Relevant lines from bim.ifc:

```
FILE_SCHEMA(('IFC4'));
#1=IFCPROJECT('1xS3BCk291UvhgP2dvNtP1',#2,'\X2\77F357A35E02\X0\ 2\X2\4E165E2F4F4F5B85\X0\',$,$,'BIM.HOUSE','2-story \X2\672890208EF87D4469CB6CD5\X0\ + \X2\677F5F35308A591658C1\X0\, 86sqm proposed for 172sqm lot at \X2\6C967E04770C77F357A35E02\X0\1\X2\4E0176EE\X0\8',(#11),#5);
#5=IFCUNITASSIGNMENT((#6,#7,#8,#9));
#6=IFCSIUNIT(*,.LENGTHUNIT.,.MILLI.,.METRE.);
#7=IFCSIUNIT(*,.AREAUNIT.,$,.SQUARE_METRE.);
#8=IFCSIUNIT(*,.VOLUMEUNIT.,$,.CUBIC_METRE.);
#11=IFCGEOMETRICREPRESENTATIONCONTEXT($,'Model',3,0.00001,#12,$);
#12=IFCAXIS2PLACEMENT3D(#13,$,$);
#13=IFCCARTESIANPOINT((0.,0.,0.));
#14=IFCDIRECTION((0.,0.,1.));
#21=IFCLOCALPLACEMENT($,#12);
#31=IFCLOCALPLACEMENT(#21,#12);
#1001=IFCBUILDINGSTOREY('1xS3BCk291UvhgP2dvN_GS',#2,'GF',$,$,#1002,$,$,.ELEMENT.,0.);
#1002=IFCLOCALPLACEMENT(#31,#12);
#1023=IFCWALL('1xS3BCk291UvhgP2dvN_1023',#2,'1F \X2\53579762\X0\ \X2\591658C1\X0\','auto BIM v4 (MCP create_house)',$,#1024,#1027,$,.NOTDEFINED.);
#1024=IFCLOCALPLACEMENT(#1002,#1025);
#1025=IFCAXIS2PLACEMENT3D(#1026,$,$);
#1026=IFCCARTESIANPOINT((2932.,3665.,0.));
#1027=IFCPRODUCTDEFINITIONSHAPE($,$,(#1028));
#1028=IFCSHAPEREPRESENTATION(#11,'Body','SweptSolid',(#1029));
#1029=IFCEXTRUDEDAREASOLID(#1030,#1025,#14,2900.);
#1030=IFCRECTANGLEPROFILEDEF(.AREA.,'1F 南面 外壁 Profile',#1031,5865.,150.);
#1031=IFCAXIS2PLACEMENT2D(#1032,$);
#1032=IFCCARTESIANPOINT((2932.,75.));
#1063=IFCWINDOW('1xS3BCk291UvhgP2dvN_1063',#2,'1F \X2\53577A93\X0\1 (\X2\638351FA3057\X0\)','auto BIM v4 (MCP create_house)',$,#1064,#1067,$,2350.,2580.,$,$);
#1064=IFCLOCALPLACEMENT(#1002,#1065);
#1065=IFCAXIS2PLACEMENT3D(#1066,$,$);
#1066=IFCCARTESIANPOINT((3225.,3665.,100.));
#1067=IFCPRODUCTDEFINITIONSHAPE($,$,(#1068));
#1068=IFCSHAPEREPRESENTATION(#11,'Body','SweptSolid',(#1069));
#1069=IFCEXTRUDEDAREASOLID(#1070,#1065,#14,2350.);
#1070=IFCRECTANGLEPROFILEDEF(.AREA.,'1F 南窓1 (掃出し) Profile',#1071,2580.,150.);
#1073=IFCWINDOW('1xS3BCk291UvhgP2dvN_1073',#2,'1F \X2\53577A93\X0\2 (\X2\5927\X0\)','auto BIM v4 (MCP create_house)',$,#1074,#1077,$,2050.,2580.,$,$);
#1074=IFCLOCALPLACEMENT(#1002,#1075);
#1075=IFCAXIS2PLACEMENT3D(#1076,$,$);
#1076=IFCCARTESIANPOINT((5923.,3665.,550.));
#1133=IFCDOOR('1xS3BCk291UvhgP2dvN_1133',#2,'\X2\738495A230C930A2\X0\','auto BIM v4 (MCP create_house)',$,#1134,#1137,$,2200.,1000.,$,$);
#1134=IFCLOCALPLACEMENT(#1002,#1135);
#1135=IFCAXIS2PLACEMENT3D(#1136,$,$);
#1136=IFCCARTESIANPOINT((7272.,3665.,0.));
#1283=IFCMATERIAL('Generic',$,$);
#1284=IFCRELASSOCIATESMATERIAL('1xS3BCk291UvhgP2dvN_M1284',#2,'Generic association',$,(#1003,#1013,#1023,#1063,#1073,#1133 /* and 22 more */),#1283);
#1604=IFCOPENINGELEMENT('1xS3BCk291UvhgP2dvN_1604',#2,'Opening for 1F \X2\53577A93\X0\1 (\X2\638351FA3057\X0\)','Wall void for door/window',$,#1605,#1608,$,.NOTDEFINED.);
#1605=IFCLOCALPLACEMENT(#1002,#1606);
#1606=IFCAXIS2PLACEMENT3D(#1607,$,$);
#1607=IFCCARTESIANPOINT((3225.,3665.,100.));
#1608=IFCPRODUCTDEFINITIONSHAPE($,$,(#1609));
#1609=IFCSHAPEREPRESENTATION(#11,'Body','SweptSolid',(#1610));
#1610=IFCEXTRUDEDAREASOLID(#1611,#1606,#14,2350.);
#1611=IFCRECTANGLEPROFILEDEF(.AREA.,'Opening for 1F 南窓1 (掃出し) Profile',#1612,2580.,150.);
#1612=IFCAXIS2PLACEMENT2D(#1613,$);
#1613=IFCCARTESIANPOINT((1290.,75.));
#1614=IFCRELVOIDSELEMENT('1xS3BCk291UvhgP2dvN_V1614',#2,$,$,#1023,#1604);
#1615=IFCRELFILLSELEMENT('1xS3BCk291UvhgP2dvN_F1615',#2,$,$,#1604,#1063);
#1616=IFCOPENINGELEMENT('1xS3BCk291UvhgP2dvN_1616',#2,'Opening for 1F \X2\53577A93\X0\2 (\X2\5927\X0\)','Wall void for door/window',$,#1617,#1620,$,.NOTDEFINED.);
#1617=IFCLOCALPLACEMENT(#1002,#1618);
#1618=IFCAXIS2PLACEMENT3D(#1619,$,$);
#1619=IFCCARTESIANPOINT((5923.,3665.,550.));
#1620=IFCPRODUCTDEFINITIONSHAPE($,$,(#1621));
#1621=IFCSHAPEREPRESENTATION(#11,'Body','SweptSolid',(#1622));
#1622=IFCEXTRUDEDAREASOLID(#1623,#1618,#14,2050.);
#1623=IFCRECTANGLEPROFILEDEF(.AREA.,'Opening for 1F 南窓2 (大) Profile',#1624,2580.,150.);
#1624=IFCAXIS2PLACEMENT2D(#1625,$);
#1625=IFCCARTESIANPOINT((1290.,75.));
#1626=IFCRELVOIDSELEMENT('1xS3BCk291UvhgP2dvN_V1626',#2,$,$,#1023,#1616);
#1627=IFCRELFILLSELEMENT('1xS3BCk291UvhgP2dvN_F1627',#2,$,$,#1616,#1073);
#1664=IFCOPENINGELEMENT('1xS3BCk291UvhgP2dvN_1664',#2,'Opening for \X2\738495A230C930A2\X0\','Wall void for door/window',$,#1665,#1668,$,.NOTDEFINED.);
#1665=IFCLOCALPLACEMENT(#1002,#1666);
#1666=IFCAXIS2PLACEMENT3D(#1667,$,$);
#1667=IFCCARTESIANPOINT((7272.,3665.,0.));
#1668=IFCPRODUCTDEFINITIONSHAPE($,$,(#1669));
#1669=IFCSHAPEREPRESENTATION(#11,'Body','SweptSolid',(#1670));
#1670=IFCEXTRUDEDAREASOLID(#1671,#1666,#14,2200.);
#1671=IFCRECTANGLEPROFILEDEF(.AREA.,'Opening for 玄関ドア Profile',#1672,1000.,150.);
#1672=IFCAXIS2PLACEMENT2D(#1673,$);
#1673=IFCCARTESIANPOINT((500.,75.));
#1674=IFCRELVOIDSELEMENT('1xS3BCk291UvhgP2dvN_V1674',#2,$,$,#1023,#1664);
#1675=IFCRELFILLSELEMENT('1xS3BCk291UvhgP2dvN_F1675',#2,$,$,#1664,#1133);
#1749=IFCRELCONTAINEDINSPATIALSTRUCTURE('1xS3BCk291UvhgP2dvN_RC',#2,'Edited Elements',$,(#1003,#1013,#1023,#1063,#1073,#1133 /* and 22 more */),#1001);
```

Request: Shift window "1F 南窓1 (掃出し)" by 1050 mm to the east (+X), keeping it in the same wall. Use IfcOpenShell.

```python
import ifcopenshell
import ifcopenshell.api.geometry
import ifcopenshell.util.placement

model = ifcopenshell.open("bim.ifc")

window = model.by_guid("1xS3BCk291UvhgP2dvN_1063")
opening = window.FillsVoids[0].RelatingOpeningElement
wall = opening.VoidsElements[0].RelatingBuildingElement

wall_matrix = ifcopenshell.util.placement.get_local_placement(wall.ObjectPlacement)
shift = wall_matrix[:3, 0] * 1050.0
before = ifcopenshell.util.placement.get_local_placement(window.ObjectPlacement)[:3, 3].copy()

# The window is not placed relative to its opening, so move both.
for product in (opening, window):
    matrix = ifcopenshell.util.placement.get_local_placement(product.ObjectPlacement)
    matrix[:3, 3] += shift
    ifcopenshell.api.geometry.edit_object_placement(model, product=product, matrix=matrix, is_si=False)

after = ifcopenshell.util.placement.get_local_placement(window.ObjectPlacement)[:3, 3]
print("window moved by", (after - before).round(3) + 0.0)

model.write("bim_edited.ifc")
```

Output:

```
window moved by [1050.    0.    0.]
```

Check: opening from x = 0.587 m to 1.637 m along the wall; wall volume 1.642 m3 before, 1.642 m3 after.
